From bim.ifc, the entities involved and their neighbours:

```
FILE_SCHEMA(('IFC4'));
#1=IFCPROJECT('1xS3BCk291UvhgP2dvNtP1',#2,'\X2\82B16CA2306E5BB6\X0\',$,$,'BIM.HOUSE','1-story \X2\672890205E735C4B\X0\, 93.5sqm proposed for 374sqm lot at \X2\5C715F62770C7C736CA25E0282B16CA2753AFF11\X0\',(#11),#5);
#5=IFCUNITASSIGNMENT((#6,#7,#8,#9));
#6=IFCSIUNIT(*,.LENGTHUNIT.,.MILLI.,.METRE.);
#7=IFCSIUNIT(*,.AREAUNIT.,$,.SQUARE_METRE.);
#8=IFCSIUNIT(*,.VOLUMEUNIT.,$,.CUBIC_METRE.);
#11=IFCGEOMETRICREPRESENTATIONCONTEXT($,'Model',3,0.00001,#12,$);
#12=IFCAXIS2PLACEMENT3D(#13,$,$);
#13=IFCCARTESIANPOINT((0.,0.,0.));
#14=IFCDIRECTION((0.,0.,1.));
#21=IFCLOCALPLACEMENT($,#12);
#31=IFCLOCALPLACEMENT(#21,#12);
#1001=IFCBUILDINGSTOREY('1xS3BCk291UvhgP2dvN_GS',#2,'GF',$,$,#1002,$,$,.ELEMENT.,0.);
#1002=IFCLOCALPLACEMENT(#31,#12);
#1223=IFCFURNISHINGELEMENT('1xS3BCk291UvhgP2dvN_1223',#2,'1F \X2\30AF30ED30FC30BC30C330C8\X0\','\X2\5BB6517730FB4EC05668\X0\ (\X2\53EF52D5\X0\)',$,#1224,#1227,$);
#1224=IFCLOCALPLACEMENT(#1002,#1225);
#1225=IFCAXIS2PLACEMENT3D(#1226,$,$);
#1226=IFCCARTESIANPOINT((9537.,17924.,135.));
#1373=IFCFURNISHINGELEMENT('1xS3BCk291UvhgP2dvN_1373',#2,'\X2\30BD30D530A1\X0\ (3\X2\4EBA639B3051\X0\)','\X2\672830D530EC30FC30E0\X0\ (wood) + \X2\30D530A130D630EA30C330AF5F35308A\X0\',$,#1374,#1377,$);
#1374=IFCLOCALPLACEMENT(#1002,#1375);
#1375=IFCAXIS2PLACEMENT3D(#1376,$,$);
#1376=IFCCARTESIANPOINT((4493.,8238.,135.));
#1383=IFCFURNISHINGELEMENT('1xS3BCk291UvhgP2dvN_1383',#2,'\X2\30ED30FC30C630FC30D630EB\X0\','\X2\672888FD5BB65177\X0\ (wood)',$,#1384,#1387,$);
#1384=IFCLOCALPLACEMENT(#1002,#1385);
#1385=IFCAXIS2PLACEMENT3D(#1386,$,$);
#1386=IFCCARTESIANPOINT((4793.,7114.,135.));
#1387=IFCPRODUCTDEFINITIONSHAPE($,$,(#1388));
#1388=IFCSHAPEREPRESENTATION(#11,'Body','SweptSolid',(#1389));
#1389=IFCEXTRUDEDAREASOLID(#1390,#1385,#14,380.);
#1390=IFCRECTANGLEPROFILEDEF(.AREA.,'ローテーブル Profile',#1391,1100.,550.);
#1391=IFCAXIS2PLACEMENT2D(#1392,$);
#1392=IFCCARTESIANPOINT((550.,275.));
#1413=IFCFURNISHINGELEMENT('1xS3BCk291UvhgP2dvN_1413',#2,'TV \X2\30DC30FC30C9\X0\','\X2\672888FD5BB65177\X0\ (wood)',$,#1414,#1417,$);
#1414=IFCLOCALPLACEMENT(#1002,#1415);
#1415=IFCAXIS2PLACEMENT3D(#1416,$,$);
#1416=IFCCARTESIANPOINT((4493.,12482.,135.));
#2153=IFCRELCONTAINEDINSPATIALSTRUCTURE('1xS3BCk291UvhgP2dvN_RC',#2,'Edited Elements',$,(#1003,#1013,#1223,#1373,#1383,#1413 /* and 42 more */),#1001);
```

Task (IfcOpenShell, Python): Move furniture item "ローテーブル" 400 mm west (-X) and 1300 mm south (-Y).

```python
import ifcopenshell
import ifcopenshell.api.geometry
import ifcopenshell.util.placement

model = ifcopenshell.open("bim.ifc")

item = model.by_id(1383)
matrix = ifcopenshell.util.placement.get_local_placement(item.ObjectPlacement)
matrix[0, 3] -= 400.0
matrix[1, 3] -= 1300.0
ifcopenshell.api.geometry.edit_object_placement(model, product=item, matrix=matrix, is_si=False)

print(ifcopenshell.util.placement.get_local_placement(item.ObjectPlacement).round(3) + 0.0)

model.write("bim_rev.ifc")
```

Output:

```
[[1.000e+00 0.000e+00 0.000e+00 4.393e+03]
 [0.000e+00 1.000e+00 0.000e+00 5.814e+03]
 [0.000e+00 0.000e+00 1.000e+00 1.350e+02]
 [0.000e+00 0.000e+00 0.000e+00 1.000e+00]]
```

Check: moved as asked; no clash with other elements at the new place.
